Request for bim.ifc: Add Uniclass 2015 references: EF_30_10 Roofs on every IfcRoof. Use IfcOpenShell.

First a look at what the model holds.

```python
import ifcopenshell

model = ifcopenshell.open("bim.ifc")
print(model.schema)
print("classifications:", [c.Name for c in model.by_type("IfcClassification")])
for ifc_class in ("IfcDoor", "IfcRoof", "IfcStair", "IfcWall", "IfcWindow"):
    print(ifc_class, len(model.by_type(ifc_class)))
```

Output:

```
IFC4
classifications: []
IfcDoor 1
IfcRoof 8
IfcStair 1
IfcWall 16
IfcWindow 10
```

```python
import ifcopenshell
import ifcopenshell.api.classification

model = ifcopenshell.open("bim.ifc")

system = ifcopenshell.api.classification.add_classification(model, classification="Uniclass 2015")

codes = {
    "IfcRoof": ("EF_30_10", "Roofs"),
}
for ifc_class, (code, name) in codes.items():
    products = model.by_type(ifc_class)
    ifcopenshell.api.classification.add_reference(
        model, products=products, classification=system, identification=code, name=name
    )
    print(code, len(products))

model.write("bim_rev.ifc")
```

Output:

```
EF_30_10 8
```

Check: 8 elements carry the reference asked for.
